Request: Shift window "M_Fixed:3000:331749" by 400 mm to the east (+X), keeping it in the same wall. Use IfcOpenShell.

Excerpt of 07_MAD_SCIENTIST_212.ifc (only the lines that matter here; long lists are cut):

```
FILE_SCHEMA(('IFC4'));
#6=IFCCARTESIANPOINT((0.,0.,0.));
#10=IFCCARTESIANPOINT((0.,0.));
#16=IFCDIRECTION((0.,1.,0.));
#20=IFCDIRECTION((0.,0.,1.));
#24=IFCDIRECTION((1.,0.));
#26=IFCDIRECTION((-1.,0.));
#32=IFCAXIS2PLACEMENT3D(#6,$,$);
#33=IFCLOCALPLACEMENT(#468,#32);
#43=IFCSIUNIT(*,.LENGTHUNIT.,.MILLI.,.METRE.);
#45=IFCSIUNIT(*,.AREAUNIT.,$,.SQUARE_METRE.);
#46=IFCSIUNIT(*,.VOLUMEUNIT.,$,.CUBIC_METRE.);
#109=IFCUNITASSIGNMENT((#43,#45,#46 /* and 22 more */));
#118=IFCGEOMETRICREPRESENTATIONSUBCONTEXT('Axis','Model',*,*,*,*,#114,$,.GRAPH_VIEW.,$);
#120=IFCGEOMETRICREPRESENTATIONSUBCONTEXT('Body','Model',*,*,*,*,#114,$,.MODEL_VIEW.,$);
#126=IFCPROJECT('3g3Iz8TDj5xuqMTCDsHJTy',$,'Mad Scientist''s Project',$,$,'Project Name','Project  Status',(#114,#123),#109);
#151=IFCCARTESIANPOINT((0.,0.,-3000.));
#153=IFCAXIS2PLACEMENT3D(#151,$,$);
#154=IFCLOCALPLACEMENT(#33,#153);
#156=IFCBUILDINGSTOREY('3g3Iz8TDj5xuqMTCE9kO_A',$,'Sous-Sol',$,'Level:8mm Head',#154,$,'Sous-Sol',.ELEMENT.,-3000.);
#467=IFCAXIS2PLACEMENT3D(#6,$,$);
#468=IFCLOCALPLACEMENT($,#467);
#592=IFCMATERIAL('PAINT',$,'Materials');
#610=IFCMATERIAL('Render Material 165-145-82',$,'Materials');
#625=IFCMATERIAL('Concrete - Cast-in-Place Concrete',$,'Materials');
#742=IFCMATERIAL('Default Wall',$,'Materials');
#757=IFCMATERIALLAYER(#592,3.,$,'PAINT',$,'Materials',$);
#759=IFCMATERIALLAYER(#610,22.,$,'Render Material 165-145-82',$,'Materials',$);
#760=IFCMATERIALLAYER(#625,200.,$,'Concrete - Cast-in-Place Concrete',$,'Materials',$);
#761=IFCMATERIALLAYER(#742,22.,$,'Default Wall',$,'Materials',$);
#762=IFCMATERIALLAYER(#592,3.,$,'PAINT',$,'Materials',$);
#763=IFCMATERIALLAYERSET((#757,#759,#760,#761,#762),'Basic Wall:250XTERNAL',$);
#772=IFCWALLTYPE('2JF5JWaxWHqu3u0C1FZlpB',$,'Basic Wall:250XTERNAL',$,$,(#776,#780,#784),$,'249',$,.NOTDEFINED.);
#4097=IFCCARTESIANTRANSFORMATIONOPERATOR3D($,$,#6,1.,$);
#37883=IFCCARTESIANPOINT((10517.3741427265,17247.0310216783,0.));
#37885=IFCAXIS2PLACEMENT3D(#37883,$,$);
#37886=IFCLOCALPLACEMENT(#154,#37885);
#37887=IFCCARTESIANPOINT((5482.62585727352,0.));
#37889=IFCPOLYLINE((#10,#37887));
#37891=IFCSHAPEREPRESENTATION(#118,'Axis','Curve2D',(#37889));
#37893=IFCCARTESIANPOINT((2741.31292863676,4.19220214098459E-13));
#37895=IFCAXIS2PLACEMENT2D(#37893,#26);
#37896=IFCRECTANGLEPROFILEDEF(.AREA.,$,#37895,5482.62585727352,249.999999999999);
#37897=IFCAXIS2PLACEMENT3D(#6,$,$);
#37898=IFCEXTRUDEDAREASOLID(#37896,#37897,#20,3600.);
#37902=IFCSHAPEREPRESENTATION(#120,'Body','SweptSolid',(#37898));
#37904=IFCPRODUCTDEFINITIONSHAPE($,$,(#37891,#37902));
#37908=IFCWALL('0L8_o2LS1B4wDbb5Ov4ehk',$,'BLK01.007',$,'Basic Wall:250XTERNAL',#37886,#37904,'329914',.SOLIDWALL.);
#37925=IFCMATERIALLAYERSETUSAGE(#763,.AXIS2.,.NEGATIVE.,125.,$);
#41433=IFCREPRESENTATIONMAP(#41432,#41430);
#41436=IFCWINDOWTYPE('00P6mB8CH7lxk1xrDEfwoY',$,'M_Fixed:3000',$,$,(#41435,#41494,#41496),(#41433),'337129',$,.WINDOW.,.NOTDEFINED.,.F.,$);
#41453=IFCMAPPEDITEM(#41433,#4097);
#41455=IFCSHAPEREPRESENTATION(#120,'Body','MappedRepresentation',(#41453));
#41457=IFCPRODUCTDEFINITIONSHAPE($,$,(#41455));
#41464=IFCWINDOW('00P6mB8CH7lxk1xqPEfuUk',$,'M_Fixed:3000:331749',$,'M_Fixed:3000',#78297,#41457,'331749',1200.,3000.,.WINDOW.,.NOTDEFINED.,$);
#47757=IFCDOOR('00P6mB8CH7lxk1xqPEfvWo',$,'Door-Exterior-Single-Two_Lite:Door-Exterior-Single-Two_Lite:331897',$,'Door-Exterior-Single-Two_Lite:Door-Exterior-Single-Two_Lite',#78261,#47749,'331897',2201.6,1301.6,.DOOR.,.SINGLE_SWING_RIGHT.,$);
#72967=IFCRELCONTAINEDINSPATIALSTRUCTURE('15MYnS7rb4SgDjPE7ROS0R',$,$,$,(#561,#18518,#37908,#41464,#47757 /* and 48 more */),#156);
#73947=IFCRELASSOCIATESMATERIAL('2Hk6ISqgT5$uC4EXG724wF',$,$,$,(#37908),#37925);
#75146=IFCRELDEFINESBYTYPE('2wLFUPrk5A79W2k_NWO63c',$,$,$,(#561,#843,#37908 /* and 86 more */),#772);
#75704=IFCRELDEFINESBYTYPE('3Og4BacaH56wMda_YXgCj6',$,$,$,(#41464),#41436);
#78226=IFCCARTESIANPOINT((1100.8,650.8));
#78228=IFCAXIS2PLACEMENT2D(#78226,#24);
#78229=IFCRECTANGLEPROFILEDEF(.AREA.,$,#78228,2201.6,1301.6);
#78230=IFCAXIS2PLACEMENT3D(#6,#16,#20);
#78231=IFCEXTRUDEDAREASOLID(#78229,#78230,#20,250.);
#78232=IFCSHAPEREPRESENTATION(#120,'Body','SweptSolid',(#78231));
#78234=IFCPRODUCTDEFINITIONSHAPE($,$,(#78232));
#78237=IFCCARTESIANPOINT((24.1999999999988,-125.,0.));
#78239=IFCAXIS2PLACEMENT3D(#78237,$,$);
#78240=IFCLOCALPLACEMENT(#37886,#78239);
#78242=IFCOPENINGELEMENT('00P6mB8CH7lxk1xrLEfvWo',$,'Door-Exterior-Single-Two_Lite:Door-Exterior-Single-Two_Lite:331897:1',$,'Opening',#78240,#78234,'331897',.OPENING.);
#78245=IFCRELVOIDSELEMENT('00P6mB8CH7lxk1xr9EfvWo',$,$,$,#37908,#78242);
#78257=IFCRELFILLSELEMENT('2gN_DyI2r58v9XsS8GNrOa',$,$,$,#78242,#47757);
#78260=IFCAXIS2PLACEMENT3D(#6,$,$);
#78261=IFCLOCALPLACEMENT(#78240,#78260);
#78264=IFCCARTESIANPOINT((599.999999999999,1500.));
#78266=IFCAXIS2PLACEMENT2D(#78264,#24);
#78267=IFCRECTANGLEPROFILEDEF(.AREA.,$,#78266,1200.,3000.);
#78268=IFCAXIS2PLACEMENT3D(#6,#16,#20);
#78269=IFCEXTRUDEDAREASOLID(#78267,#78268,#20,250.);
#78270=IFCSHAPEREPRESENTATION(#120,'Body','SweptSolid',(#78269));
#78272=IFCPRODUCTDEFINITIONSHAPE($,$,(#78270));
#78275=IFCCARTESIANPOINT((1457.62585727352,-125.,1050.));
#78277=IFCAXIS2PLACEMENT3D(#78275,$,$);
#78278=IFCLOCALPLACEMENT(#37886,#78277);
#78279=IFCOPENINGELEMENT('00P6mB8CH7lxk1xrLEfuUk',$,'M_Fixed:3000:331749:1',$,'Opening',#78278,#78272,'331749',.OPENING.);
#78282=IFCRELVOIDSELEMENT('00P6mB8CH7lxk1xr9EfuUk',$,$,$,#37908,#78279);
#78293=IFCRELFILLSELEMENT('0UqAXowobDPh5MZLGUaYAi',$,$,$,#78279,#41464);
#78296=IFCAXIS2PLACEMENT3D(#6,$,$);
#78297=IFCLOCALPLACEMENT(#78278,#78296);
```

```python
import ifcopenshell
import ifcopenshell.api.geometry
import ifcopenshell.util.placement

model = ifcopenshell.open("07_MAD_SCIENTIST_212.ifc")

window = model.by_guid("00P6mB8CH7lxk1xqPEfuUk")
opening = window.FillsVoids[0].RelatingOpeningElement
wall = opening.VoidsElements[0].RelatingBuildingElement

wall_matrix = ifcopenshell.util.placement.get_local_placement(wall.ObjectPlacement)
shift = wall_matrix[:3, 0] * 400.0
before = ifcopenshell.util.placement.get_local_placement(window.ObjectPlacement)[:3, 3].copy()

# The window is placed relative to its opening, so it follows when the opening moves.
matrix = ifcopenshell.util.placement.get_local_placement(opening.ObjectPlacement)
matrix[:3, 3] += shift
ifcopenshell.api.geometry.edit_object_placement(
    model, product=opening, matrix=matrix, is_si=False, should_transform_children=True
)

after = ifcopenshell.util.placement.get_local_placement(window.ObjectPlacement)[:3, 3]
print("window moved by", (after - before).round(3) + 0.0)

model.write("07_MAD_SCIENTIST_212_rev.ifc")
```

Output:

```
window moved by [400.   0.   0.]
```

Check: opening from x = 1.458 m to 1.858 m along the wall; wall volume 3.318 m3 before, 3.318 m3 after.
